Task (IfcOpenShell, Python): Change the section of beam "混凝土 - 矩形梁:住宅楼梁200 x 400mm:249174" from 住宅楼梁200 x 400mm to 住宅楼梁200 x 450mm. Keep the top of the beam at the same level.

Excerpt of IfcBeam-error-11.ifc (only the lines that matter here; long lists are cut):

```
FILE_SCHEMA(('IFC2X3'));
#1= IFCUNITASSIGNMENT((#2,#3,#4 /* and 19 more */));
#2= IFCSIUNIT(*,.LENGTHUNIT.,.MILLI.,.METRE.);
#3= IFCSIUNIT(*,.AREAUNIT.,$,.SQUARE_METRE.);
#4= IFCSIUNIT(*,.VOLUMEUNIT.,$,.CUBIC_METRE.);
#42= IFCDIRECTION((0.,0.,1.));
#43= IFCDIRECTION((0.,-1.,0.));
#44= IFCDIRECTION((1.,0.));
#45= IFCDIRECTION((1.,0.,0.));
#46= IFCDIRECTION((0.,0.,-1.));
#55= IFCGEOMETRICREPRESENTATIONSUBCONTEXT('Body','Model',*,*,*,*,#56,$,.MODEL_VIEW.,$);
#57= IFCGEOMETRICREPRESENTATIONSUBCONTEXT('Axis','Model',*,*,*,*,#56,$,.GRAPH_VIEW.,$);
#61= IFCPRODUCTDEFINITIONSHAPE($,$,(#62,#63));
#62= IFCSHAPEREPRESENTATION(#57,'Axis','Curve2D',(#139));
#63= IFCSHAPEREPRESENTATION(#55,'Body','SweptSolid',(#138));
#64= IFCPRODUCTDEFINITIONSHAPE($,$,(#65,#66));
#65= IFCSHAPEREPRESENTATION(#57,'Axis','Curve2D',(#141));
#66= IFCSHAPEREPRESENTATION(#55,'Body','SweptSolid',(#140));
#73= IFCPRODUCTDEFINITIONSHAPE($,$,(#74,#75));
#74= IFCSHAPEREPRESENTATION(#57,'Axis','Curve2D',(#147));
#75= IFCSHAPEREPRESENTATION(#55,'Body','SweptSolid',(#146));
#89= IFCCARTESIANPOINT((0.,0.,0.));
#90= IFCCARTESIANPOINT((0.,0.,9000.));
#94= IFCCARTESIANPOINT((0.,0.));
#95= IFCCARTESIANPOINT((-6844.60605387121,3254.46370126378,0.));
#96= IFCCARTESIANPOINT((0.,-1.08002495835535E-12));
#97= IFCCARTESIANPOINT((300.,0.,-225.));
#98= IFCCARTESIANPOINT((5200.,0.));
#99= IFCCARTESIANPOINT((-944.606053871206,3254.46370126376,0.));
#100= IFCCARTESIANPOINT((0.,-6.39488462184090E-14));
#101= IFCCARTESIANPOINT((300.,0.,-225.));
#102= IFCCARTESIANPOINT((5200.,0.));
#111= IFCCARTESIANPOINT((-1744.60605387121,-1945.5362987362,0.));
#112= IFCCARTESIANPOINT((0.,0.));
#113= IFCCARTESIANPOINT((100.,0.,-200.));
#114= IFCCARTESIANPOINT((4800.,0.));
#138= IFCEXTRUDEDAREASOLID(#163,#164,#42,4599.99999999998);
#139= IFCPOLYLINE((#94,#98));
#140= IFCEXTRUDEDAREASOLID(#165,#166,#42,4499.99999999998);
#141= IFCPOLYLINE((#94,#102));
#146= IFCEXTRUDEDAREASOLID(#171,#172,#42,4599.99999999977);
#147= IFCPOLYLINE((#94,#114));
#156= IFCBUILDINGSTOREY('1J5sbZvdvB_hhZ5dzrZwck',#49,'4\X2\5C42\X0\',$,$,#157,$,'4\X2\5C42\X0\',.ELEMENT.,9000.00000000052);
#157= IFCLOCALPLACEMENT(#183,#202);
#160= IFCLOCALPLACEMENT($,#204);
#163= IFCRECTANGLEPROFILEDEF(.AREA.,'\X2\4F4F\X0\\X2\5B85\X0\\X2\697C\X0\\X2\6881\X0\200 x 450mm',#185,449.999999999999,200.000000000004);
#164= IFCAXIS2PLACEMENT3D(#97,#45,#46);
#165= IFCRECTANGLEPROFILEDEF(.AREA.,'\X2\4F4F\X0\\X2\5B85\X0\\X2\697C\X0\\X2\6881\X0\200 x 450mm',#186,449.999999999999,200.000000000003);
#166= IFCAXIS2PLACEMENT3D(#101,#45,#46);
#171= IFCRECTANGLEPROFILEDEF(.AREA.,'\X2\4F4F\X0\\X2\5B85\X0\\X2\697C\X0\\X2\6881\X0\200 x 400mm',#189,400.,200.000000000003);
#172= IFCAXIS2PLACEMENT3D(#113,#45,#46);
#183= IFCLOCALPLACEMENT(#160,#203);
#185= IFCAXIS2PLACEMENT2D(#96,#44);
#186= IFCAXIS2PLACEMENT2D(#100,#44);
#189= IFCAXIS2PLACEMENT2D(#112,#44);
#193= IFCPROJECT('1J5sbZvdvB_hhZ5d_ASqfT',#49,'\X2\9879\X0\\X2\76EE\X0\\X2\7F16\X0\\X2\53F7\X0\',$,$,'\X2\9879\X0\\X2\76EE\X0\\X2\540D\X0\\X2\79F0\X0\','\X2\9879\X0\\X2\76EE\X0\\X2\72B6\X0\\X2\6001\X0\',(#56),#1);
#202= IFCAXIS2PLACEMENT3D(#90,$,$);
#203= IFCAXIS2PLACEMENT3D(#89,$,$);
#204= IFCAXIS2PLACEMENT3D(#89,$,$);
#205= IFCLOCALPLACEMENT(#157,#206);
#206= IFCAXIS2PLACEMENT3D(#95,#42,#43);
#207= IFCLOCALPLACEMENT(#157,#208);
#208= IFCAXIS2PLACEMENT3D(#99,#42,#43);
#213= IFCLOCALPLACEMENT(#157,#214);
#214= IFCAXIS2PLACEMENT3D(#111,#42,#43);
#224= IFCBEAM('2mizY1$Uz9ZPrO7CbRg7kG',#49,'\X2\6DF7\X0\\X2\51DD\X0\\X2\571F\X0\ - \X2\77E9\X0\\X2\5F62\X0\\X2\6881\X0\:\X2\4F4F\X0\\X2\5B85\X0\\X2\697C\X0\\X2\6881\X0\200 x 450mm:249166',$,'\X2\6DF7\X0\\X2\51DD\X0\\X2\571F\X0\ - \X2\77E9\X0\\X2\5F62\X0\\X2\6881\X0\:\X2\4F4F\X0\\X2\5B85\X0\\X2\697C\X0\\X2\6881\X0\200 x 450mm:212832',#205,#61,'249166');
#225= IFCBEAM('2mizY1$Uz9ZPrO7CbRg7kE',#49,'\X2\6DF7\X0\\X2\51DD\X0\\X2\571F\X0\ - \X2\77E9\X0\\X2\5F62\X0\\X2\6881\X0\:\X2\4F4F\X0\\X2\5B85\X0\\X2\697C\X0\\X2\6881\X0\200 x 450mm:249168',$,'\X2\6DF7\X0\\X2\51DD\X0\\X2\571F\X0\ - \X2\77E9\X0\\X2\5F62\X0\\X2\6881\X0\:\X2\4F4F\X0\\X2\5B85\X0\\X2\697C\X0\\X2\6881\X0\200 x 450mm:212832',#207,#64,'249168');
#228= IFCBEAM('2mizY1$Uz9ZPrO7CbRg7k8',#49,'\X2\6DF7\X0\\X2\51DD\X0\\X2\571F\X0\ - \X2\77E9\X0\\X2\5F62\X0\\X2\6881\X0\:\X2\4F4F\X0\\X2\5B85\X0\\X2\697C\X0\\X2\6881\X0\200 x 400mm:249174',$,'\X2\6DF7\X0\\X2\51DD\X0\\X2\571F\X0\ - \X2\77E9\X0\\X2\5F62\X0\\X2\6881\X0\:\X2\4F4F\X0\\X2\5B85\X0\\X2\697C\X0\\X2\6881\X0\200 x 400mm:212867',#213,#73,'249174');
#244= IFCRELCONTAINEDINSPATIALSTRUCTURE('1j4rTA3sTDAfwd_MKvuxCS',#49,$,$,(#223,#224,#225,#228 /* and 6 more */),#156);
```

```python
import ifcopenshell
import ifcopenshell.util.element
import ifcopenshell.util.representation

model = ifcopenshell.open("IfcBeam-error-11.ifc")

member = model.by_guid("2mizY1$Uz9ZPrO7CbRg7k8")
source = next(p for p in model.by_type("IfcRectangleProfileDef") if p.ProfileName == "住宅楼梁200 x 450mm")

body = ifcopenshell.util.representation.get_representation(member, "Model", "Body")
solid = body.Items[0]
old_profile = solid.SweptArea

# Copy the section's sizes but keep this member's own profile position.
profile = ifcopenshell.util.element.copy(model, source)
# Profiles are centred, so shift by half the change in depth to hold the top.
shift = (old_profile.XDim - profile.XDim) / 2
x, y = old_profile.Position.Location.Coordinates
up = (-1.0, 0.0)  # upwards, in the solid's own plane
location = model.createIfcCartesianPoint((x + up[0] * shift, y + up[1] * shift))
profile.Position = model.createIfcAxis2Placement2D(location, old_profile.Position.RefDirection)
solid.SweptArea = profile
if not model.get_total_inverses(old_profile):
    ifcopenshell.util.element.remove_deep2(model, old_profile)
member.Name = member.Name.replace("住宅楼梁200 x 400mm", "住宅楼梁200 x 450mm")
member.ObjectType = member.ObjectType.replace("住宅楼梁200 x 400mm", "住宅楼梁200 x 450mm")

print(solid.SweptArea)

model.write("IfcBeam-error-11_v2.ifc")
```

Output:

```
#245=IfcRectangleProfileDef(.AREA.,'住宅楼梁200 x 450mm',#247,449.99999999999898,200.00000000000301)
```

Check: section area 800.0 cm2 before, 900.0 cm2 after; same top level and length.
